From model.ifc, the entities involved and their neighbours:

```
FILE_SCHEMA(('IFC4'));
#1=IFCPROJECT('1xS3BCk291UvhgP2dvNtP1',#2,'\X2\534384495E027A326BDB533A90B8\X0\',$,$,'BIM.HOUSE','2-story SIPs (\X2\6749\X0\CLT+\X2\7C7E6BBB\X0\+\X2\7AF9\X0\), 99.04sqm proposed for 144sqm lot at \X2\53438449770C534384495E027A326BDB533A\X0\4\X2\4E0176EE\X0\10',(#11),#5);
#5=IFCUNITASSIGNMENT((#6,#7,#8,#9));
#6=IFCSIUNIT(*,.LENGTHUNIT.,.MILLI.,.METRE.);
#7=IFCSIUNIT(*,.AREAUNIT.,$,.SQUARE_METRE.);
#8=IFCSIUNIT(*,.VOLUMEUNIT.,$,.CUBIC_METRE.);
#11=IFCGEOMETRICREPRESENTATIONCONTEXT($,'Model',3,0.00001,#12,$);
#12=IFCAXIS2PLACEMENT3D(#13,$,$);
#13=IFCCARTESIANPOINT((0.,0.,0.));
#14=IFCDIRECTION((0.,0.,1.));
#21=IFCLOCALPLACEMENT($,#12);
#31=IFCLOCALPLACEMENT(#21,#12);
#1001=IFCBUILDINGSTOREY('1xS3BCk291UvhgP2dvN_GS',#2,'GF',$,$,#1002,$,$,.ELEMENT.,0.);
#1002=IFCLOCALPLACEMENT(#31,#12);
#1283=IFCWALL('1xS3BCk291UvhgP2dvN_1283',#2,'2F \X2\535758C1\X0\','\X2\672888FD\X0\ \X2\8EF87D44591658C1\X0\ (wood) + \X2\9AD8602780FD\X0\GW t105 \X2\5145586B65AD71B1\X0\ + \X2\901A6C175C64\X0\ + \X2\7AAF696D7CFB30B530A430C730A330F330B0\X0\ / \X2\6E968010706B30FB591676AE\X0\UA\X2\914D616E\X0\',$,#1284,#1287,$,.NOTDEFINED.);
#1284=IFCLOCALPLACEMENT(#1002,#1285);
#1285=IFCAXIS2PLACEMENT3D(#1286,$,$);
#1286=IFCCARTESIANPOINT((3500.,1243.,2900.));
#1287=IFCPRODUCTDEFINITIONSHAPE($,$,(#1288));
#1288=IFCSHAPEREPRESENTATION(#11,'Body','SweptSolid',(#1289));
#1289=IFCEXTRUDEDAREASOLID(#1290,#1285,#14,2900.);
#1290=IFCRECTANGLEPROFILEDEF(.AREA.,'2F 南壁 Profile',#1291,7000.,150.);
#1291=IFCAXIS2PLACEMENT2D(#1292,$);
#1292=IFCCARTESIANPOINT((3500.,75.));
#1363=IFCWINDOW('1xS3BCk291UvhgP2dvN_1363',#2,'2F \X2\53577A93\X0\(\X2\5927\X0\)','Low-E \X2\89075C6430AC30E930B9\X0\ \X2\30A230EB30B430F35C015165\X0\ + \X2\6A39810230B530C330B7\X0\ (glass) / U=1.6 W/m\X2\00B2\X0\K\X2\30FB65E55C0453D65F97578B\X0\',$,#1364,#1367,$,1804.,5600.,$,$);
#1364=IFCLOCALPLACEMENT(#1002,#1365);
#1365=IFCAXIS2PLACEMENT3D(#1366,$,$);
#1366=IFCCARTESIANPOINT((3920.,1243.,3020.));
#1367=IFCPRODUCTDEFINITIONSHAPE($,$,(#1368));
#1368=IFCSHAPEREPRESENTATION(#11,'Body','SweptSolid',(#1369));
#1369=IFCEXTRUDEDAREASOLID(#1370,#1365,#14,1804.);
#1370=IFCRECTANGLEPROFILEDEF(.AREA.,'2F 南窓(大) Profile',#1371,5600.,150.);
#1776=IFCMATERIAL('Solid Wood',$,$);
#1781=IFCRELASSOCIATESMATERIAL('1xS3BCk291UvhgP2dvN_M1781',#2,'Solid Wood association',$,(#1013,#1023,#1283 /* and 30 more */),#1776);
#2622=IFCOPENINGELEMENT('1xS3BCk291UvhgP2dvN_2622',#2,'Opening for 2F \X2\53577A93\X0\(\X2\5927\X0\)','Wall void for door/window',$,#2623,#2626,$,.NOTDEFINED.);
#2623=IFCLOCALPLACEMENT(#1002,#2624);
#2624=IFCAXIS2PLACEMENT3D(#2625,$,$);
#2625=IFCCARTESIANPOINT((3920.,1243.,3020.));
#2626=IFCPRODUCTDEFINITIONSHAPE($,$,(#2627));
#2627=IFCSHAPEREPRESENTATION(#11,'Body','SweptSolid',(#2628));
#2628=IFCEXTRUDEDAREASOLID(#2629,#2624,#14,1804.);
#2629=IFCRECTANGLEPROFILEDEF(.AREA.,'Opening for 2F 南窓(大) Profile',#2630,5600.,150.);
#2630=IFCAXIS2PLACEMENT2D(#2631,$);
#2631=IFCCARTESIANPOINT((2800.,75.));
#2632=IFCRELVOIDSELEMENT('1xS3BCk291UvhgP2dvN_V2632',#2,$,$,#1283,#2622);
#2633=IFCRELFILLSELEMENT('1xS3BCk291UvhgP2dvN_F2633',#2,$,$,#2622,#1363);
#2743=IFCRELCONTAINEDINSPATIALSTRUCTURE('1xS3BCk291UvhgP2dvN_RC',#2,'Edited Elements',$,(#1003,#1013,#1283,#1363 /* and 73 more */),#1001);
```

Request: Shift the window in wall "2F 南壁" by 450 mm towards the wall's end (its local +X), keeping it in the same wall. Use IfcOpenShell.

```python
import ifcopenshell
import ifcopenshell.api.geometry
import ifcopenshell.util.placement
import ifcopenshell.util.unit

model = ifcopenshell.open("model.ifc")
unit_scale = ifcopenshell.util.unit.calculate_unit_scale(model)

window = model.by_guid("1xS3BCk291UvhgP2dvN_1363")
opening = window.FillsVoids[0].RelatingOpeningElement
wall = opening.VoidsElements[0].RelatingBuildingElement

wall_matrix = ifcopenshell.util.placement.get_local_placement(wall.ObjectPlacement)
shift = wall_matrix[:3, 0] * 0.45 / unit_scale
before = ifcopenshell.util.placement.get_local_placement(window.ObjectPlacement)[:3, 3].copy()

# The window is not placed relative to its opening, so move both.
for product in (opening, window):
    matrix = ifcopenshell.util.placement.get_local_placement(product.ObjectPlacement)
    matrix[:3, 3] += shift
    ifcopenshell.api.geometry.edit_object_placement(model, product=product, matrix=matrix, is_si=False)

after = ifcopenshell.util.placement.get_local_placement(window.ObjectPlacement)[:3, 3]
print("window moved by", (after - before).round(3) + 0.0)

model.write("model_rev.ifc")
```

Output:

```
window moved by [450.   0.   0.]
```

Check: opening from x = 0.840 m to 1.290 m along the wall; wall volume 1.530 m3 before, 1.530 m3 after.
